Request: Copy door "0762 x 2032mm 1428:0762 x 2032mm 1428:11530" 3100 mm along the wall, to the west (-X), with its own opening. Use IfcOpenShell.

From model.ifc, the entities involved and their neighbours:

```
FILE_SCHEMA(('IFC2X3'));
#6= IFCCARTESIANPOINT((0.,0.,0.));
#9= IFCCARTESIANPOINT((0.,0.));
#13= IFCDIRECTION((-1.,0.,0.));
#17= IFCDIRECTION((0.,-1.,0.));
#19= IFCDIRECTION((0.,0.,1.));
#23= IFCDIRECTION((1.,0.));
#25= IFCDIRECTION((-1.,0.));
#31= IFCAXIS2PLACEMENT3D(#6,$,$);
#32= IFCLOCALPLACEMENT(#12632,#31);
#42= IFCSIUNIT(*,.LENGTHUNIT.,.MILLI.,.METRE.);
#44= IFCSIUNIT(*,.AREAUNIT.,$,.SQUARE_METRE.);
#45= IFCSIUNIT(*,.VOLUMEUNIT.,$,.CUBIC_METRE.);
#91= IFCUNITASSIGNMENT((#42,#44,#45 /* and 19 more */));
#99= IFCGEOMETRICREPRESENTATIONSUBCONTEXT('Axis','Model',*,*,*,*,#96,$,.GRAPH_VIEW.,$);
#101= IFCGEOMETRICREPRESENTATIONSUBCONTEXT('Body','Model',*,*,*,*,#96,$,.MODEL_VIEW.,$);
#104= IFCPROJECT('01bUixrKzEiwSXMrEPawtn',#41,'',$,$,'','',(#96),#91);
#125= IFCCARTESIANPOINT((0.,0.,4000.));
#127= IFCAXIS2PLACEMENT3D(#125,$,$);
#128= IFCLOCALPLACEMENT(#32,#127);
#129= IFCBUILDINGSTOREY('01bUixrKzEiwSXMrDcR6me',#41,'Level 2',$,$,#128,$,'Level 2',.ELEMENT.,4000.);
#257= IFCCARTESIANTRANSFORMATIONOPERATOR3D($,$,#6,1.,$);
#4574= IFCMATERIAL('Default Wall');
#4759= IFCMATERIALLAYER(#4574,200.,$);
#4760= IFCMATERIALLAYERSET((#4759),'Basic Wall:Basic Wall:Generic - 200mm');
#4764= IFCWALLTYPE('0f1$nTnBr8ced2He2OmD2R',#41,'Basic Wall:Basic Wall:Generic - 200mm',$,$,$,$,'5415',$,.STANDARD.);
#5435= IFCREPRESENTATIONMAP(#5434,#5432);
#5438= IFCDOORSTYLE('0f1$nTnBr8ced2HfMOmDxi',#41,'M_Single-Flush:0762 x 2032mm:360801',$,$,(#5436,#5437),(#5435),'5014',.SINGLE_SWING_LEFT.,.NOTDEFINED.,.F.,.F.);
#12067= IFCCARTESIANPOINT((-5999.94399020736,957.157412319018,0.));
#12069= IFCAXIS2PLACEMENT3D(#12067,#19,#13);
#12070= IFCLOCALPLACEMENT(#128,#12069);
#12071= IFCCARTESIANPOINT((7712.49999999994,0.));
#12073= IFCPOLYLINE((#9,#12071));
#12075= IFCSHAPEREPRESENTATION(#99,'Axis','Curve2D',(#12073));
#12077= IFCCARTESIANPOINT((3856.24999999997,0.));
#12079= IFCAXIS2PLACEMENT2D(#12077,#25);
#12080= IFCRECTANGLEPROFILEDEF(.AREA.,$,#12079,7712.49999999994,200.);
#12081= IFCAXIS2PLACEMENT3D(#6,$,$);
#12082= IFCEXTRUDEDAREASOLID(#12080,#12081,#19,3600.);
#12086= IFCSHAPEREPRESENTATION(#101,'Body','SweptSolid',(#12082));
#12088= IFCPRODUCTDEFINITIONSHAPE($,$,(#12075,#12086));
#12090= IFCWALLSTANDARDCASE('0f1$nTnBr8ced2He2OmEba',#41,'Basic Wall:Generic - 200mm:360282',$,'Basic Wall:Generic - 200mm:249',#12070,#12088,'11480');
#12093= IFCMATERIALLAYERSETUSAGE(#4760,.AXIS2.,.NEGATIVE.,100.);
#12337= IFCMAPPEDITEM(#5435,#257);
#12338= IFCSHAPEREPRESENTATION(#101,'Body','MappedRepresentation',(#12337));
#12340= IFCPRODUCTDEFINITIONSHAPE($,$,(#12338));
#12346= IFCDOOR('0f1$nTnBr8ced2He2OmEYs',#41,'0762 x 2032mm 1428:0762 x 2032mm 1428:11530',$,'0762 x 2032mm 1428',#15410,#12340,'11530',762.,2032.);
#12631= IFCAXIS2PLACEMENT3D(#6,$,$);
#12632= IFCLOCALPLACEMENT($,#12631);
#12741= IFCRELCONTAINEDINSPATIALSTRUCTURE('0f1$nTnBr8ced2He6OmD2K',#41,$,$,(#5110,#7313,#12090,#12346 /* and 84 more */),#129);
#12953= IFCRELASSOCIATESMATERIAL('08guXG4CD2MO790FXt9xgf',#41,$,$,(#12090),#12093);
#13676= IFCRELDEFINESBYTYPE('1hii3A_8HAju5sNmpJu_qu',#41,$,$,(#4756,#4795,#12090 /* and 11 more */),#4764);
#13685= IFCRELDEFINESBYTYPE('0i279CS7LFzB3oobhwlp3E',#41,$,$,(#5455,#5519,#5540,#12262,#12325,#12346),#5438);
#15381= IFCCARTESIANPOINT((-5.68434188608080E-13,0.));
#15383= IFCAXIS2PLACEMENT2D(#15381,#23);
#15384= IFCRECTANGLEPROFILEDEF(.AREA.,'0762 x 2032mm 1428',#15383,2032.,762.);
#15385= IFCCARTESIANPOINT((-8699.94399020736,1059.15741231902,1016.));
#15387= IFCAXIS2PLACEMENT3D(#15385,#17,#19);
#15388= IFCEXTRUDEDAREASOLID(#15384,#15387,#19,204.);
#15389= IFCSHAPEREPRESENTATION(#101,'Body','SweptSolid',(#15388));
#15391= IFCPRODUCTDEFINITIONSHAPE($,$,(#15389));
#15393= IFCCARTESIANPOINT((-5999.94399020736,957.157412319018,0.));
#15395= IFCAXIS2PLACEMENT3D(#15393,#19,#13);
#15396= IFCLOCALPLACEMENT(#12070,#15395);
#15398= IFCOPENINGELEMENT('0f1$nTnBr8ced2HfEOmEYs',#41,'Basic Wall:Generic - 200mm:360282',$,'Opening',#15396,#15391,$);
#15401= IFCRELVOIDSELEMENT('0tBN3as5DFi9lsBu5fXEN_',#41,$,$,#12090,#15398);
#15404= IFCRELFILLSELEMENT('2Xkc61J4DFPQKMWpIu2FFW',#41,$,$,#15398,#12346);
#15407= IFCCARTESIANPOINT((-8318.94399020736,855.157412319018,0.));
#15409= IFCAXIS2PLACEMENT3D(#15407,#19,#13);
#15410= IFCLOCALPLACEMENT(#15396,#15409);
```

```python
import ifcopenshell
import ifcopenshell.api.feature
import ifcopenshell.api.geometry
import ifcopenshell.api.root
import ifcopenshell.geom
import ifcopenshell.util.element
import ifcopenshell.util.placement
import ifcopenshell.util.shape

model = ifcopenshell.open("model.ifc")
settings = ifcopenshell.geom.settings()


def volume(element):
    """Net volume in cubic metres, openings subtracted."""
    shape = ifcopenshell.geom.create_shape(settings, element)
    return ifcopenshell.util.shape.get_volume(shape.geometry)


def reuse_history(source, copy):
    """copy_class also copies each property set's owner history, people and application; keep the originals."""
    for rel in copy.IsDefinedBy:
        if rel.is_a("IfcRelDefinesByProperties") and (history := rel.RelatingPropertyDefinition.OwnerHistory):
            rel.RelatingPropertyDefinition.OwnerHistory = source.OwnerHistory
            ifcopenshell.util.element.remove_deep2(model, history)


door = model.by_id(12346)
opening = door.FillsVoids[0].RelatingOpeningElement
wall = opening.VoidsElements[0].RelatingBuildingElement
before = volume(wall)
shift = ifcopenshell.util.placement.get_local_placement(wall.ObjectPlacement)[:3, 0] * 3100.0

# copy_class copies the void relationship, type, container and properties, but no geometry.
new_opening = ifcopenshell.api.root.copy_class(model, product=opening)
new_opening.Representation = ifcopenshell.util.element.copy_deep(
    model, opening.Representation, exclude=["IfcGeometricRepresentationContext", "IfcRepresentationMap"]
)
new_opening.Name = "Basic Wall:Generic - 200mm"
new_door = ifcopenshell.api.root.copy_class(model, product=door)
new_door.Representation = ifcopenshell.util.element.copy_deep(
    model, door.Representation, exclude=["IfcGeometricRepresentationContext", "IfcRepresentationMap"]
)
new_door.Name = "0762 x 2032mm 1428:0762 x 2032mm 1428"
new_door.Tag = None
reuse_history(door, new_door)
fills = ifcopenshell.api.feature.add_filling(model, opening=new_opening, element=new_door)
fills.OwnerHistory = new_door.OwnerHistory  # required in IFC2X3

for old, new in ((opening, new_opening), (door, new_door)):
    matrix = ifcopenshell.util.placement.get_local_placement(old.ObjectPlacement)
    matrix[:3, 3] += shift
    ifcopenshell.api.geometry.edit_object_placement(model, product=new, matrix=matrix, is_si=False)

after = volume(wall)

print(f"wall volume {before:.3f} -> {after:.3f} m3")

model.write("model_updated.ifc")
```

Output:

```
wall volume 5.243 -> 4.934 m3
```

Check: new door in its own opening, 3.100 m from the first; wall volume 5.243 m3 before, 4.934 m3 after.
